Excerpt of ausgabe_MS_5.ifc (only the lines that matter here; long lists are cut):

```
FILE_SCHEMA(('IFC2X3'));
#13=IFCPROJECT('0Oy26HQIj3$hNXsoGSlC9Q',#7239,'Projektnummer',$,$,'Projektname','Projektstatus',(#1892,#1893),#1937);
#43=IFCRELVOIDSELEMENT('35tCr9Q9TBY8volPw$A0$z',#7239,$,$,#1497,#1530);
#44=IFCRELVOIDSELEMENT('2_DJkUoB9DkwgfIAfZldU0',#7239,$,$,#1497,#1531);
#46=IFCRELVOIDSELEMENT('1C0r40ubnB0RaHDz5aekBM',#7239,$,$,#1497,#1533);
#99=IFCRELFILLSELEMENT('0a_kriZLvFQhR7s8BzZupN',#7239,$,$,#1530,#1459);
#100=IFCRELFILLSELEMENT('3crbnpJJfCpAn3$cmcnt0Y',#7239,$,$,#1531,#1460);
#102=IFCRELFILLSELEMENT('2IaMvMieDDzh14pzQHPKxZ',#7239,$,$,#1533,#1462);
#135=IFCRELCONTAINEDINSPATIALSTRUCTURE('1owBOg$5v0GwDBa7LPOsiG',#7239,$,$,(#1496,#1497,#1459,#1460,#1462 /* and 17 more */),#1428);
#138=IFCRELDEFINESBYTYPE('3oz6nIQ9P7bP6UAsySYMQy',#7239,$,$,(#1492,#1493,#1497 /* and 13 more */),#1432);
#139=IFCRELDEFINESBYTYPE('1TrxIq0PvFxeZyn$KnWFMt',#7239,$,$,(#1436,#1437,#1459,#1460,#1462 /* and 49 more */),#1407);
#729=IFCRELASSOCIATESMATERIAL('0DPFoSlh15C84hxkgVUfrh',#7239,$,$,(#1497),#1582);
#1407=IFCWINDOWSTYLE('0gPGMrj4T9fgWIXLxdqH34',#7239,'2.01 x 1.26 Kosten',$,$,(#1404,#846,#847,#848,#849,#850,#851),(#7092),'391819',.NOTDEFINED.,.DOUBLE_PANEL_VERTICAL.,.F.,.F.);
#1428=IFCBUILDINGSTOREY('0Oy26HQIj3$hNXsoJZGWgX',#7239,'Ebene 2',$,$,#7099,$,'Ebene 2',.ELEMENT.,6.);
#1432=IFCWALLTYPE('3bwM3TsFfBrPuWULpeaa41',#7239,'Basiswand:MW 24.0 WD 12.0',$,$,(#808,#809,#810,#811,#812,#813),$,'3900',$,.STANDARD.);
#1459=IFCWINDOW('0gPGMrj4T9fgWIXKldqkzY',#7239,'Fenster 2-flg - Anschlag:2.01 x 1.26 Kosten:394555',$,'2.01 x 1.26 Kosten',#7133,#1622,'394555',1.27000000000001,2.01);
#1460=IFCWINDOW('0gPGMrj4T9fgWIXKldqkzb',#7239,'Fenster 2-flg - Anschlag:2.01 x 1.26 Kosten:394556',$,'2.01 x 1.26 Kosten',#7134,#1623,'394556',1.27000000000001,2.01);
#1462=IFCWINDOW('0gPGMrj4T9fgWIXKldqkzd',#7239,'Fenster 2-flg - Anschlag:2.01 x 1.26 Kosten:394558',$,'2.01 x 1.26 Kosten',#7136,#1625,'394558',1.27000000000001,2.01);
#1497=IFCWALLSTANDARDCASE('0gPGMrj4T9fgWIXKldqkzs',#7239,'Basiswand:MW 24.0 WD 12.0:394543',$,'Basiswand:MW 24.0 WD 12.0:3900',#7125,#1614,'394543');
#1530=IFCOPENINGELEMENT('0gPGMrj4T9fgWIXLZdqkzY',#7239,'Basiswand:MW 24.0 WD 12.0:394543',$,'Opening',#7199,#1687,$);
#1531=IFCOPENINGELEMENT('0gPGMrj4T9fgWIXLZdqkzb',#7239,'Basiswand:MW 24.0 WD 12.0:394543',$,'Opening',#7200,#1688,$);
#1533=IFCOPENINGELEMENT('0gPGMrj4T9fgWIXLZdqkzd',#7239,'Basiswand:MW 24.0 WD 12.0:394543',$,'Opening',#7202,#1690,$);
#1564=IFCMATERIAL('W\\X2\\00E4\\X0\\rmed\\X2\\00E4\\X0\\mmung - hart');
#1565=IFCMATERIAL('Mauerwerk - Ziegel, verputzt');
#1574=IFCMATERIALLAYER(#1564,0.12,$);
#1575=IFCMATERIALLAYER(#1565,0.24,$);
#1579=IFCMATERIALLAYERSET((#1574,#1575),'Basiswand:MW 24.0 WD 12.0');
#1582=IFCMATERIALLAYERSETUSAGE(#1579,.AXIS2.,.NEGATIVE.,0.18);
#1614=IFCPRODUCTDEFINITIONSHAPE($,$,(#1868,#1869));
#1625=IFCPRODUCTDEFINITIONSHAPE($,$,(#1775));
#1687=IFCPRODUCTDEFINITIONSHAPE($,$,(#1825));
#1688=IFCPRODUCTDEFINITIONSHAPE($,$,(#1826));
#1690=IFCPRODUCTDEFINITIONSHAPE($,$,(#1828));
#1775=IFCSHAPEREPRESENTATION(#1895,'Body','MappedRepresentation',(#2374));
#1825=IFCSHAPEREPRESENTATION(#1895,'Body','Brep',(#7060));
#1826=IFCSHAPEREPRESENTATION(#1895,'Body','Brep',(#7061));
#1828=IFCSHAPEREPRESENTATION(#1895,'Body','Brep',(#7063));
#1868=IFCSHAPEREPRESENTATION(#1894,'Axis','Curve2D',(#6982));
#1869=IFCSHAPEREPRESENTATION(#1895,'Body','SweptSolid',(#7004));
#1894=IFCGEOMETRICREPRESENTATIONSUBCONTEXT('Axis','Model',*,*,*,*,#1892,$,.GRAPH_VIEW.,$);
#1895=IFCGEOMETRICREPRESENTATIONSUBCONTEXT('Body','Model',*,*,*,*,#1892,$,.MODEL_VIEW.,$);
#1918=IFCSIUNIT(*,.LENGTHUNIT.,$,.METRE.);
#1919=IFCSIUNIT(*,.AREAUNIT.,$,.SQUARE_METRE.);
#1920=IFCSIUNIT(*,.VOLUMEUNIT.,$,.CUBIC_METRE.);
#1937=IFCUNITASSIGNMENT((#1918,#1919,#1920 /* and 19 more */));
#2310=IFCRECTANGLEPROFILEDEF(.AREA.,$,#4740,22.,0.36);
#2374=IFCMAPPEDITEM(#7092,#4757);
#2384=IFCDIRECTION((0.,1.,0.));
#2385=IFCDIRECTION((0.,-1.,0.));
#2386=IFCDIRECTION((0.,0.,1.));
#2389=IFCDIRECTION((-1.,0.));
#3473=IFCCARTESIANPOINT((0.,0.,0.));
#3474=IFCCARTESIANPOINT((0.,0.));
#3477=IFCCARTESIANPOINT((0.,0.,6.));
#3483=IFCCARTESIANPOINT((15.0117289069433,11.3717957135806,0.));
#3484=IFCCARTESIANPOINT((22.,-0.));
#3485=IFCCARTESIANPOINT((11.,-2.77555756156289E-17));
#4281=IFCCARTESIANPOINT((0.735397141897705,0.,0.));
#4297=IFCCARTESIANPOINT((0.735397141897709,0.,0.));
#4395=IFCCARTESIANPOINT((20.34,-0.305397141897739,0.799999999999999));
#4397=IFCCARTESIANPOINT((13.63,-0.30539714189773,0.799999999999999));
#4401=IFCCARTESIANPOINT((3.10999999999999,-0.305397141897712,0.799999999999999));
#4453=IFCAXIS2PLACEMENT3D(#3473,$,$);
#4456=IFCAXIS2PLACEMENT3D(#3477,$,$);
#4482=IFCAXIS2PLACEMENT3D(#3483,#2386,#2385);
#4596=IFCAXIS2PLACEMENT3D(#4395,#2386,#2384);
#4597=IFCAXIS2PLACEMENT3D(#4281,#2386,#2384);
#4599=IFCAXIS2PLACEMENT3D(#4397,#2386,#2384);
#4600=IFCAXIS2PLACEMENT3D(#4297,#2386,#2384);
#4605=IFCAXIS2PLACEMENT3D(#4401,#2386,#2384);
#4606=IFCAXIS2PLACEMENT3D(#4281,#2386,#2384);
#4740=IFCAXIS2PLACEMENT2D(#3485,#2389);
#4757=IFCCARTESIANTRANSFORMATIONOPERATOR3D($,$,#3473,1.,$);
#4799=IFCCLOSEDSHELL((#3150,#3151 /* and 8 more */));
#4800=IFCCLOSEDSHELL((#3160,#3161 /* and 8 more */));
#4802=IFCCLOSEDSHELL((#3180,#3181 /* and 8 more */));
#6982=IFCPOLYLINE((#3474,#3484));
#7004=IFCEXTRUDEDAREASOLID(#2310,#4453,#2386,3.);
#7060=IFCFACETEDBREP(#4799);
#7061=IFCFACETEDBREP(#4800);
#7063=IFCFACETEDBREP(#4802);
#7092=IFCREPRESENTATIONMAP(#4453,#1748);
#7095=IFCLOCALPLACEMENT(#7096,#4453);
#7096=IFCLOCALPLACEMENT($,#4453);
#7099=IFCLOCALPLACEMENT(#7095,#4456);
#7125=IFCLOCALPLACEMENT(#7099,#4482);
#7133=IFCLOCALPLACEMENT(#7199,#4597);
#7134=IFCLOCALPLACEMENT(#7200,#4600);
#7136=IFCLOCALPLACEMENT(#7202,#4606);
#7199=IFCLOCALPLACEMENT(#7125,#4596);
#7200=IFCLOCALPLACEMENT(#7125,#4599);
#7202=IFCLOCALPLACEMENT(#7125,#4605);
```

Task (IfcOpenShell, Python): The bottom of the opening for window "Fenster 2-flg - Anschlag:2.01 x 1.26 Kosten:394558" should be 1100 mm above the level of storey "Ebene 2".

```python
import numpy as np
import ifcopenshell
import ifcopenshell.api.geometry
import ifcopenshell.geom
import ifcopenshell.util.element
import ifcopenshell.util.placement
import ifcopenshell.util.shape
import ifcopenshell.util.unit

model = ifcopenshell.open("ausgabe_MS_5.ifc")
unit_scale = ifcopenshell.util.unit.calculate_unit_scale(model)

window = model.by_id(1462)
opening = window.FillsVoids[0].RelatingOpeningElement
storey = ifcopenshell.util.element.get_container(window, ifc_class="IfcBuildingStorey")
level = ifcopenshell.util.placement.get_local_placement(storey.ObjectPlacement)[2, 3]

# The opening's origin need not be at the sill, so measure its lowest point.
shape = ifcopenshell.geom.create_shape(ifcopenshell.geom.settings(), opening)
bottom = ifcopenshell.util.shape.get_shape_bottom_elevation(shape, shape.geometry) / unit_scale
dz = level + 1.1 / unit_scale - bottom

shift = np.array([0.0, 0.0, dz])
# The window is placed relative to its opening, so it follows when the opening moves.
matrix = ifcopenshell.util.placement.get_local_placement(opening.ObjectPlacement)
matrix[:3, 3] += shift
ifcopenshell.api.geometry.edit_object_placement(
    model, product=opening, matrix=matrix, is_si=False, should_transform_children=True
)

print(f"moved by {dz * unit_scale:+.3f} m")

model.write("ausgabe_MS_5_updated.ifc")
```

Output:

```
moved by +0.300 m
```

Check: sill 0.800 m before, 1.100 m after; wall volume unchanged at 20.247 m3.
